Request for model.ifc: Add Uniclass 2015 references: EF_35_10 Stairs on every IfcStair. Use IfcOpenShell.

First a look at what the model holds.

```python
import ifcopenshell

model = ifcopenshell.open("model.ifc")
print(model.schema)
print("classifications:", [c.Name for c in model.by_type("IfcClassification")])
for ifc_class in ("IfcDoor", "IfcRoof", "IfcStair", "IfcWall", "IfcWindow"):
    print(ifc_class, len(model.by_type(ifc_class)))
```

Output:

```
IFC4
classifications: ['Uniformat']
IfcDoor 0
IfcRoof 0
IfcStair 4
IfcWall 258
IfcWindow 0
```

```python
import ifcopenshell
import ifcopenshell.api.classification

model = ifcopenshell.open("model.ifc")

system = ifcopenshell.api.classification.add_classification(model, classification="Uniclass 2015")

codes = {
    "IfcStair": ("EF_35_10", "Stairs"),
}
for ifc_class, (code, name) in codes.items():
    products = model.by_type(ifc_class)
    ifcopenshell.api.classification.add_reference(
        model, products=products, classification=system, identification=code, name=name
    )
    print(code, len(products))

model.write("model_edited.ifc")
```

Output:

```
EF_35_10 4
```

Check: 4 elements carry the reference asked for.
